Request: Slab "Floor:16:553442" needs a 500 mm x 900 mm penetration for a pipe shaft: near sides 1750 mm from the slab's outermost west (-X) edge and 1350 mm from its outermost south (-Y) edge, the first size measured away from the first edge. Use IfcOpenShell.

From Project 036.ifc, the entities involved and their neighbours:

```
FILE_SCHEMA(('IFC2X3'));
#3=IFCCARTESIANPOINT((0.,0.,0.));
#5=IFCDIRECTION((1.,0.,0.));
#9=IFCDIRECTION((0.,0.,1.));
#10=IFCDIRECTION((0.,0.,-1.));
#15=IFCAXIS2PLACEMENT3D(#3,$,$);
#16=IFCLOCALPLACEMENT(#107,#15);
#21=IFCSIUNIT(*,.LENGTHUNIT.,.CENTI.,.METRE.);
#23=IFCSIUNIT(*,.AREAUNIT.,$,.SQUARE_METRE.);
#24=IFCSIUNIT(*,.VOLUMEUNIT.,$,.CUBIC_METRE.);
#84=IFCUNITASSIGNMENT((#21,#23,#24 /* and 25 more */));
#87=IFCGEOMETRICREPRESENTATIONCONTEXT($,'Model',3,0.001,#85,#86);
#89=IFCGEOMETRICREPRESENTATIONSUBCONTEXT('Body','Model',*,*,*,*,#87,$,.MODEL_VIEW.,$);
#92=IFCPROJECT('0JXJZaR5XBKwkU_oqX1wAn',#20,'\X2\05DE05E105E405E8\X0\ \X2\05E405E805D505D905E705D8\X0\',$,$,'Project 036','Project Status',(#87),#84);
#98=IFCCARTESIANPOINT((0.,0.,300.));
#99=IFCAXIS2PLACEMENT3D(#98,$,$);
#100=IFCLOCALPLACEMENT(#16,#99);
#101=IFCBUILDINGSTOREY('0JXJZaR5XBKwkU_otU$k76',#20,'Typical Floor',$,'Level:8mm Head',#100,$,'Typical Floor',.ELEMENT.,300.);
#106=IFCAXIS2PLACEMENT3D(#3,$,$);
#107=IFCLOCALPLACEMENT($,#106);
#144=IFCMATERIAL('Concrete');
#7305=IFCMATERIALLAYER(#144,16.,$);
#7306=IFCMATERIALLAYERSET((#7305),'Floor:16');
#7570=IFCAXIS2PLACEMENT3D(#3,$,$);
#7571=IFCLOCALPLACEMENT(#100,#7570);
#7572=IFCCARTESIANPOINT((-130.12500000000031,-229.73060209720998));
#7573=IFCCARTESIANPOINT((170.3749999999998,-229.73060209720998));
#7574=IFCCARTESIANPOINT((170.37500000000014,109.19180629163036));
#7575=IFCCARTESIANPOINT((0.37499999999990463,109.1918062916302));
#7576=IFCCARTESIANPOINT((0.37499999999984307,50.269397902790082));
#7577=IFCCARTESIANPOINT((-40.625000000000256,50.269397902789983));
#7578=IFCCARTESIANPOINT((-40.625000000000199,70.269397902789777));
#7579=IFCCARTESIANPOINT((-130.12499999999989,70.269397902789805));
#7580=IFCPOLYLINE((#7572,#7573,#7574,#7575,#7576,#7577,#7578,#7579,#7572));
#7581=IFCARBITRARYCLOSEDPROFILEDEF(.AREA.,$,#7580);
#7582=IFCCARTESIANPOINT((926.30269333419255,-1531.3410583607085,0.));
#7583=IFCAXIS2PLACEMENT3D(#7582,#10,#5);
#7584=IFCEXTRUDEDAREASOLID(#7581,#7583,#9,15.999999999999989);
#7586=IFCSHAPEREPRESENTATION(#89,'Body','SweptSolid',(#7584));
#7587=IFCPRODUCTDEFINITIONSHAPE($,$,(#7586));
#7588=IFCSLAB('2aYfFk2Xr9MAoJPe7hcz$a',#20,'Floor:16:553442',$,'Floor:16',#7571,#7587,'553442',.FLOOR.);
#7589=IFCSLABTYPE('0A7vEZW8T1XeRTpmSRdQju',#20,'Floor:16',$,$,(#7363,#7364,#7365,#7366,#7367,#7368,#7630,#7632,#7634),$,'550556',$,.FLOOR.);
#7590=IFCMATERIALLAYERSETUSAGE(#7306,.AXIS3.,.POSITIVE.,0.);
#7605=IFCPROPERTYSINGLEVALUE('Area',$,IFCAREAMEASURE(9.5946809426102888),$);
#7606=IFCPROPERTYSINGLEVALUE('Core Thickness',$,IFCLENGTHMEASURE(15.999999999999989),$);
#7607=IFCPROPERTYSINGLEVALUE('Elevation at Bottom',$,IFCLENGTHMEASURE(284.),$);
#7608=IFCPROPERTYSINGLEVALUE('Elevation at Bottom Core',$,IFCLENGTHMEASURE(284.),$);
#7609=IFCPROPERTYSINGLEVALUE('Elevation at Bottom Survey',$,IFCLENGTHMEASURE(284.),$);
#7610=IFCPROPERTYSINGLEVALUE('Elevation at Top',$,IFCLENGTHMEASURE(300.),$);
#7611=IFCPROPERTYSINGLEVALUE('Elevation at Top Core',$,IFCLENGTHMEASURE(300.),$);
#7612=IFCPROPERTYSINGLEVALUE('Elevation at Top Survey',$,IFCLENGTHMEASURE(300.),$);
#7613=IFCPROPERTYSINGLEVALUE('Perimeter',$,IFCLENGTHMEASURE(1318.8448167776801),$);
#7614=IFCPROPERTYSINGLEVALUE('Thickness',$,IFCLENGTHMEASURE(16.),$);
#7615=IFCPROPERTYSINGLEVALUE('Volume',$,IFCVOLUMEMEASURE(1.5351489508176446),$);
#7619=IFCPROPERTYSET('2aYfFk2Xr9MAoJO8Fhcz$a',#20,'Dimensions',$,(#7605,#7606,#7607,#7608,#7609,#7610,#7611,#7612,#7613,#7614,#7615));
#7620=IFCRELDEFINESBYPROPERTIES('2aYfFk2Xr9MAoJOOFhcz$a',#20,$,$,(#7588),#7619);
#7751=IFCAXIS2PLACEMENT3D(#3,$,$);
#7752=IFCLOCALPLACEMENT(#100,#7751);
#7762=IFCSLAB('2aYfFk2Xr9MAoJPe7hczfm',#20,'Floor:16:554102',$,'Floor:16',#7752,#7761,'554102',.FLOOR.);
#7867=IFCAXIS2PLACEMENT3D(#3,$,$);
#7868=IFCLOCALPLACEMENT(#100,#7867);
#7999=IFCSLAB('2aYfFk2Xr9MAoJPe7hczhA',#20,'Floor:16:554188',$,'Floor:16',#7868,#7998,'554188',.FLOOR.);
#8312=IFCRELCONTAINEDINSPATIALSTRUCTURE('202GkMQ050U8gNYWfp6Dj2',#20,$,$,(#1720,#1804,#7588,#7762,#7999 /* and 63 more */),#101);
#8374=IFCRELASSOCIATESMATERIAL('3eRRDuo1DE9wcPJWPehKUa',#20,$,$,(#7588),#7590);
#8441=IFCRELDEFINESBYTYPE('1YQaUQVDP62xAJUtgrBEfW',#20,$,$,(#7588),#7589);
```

```python
import numpy as np
import ifcopenshell
import ifcopenshell.api.feature
import ifcopenshell.api.geometry
import ifcopenshell.api.pset
import ifcopenshell.api.root
import ifcopenshell.geom
import ifcopenshell.util.element
import ifcopenshell.util.placement
import ifcopenshell.util.representation
import ifcopenshell.util.shape
import ifcopenshell.util.unit

model = ifcopenshell.open("Project 036.ifc")
unit_scale = ifcopenshell.util.unit.calculate_unit_scale(model)
area_scale = ifcopenshell.util.unit.calculate_unit_scale(model, "AREAUNIT")
volume_scale = ifcopenshell.util.unit.calculate_unit_scale(model, "VOLUMEUNIT")
settings = ifcopenshell.geom.settings()


def volume(element):
    """Net volume in cubic metres, openings subtracted."""
    shape = ifcopenshell.geom.create_shape(settings, element)
    return ifcopenshell.util.shape.get_volume(shape.geometry)


slab = model.by_guid("2aYfFk2Xr9MAoJPe7hcz$a")
before = volume(slab)

# Extent in the slab's own axes, in metres. The edges named are its -X and -Y sides.
slab_shape = ifcopenshell.geom.create_shape(settings, slab)
vertices = ifcopenshell.util.shape.get_vertices(slab_shape.geometry)
x_min, y_min, bottom = vertices.min(axis=0)
top = vertices[:, 2].max()

opening = ifcopenshell.api.root.create_entity(model, ifc_class="IfcOpeningElement", name="Pipe shaft opening")
context = ifcopenshell.util.representation.get_context(model, "Model", "Body", "MODEL_VIEW")
width, depth = 0.5, 0.9
outline = [(0.0, 0.0), (width, 0.0), (width, depth), (0.0, depth), (0.0, 0.0)]
# Overshoot both faces by 50 mm so the cut is clean.
shape = ifcopenshell.api.geometry.add_slab_representation(
    model, context=context, depth=top - bottom + 0.1, polyline=outline
)
ifcopenshell.api.geometry.assign_representation(model, product=opening, representation=shape)

matrix = ifcopenshell.util.placement.get_local_placement(slab.ObjectPlacement)
matrix[:, 3] = matrix @ np.append(np.array([x_min + 1.75, y_min + 1.35, bottom - 0.05]) / unit_scale, 1.0)
ifcopenshell.api.geometry.edit_object_placement(model, product=opening, matrix=matrix, is_si=False)
ifcopenshell.api.feature.add_feature(model, feature=opening, element=slab)

after = volume(slab)

# Update the slab's stored quantities.
pset = model.by_id(ifcopenshell.util.element.get_pset(slab, "Dimensions", should_inherit=False)["id"])
ifcopenshell.api.pset.edit_pset(model, pset=pset, properties={
    "Area": model.create_entity("IfcAreaMeasure", after / (top - bottom) / area_scale),
    "Volume": model.create_entity("IfcVolumeMeasure", after / volume_scale),
})

print(f"slab volume {before:.3f} -> {after:.3f} m3")

model.write("Project 036_edited.ifc")
```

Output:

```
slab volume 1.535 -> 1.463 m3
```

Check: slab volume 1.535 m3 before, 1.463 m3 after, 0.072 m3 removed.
